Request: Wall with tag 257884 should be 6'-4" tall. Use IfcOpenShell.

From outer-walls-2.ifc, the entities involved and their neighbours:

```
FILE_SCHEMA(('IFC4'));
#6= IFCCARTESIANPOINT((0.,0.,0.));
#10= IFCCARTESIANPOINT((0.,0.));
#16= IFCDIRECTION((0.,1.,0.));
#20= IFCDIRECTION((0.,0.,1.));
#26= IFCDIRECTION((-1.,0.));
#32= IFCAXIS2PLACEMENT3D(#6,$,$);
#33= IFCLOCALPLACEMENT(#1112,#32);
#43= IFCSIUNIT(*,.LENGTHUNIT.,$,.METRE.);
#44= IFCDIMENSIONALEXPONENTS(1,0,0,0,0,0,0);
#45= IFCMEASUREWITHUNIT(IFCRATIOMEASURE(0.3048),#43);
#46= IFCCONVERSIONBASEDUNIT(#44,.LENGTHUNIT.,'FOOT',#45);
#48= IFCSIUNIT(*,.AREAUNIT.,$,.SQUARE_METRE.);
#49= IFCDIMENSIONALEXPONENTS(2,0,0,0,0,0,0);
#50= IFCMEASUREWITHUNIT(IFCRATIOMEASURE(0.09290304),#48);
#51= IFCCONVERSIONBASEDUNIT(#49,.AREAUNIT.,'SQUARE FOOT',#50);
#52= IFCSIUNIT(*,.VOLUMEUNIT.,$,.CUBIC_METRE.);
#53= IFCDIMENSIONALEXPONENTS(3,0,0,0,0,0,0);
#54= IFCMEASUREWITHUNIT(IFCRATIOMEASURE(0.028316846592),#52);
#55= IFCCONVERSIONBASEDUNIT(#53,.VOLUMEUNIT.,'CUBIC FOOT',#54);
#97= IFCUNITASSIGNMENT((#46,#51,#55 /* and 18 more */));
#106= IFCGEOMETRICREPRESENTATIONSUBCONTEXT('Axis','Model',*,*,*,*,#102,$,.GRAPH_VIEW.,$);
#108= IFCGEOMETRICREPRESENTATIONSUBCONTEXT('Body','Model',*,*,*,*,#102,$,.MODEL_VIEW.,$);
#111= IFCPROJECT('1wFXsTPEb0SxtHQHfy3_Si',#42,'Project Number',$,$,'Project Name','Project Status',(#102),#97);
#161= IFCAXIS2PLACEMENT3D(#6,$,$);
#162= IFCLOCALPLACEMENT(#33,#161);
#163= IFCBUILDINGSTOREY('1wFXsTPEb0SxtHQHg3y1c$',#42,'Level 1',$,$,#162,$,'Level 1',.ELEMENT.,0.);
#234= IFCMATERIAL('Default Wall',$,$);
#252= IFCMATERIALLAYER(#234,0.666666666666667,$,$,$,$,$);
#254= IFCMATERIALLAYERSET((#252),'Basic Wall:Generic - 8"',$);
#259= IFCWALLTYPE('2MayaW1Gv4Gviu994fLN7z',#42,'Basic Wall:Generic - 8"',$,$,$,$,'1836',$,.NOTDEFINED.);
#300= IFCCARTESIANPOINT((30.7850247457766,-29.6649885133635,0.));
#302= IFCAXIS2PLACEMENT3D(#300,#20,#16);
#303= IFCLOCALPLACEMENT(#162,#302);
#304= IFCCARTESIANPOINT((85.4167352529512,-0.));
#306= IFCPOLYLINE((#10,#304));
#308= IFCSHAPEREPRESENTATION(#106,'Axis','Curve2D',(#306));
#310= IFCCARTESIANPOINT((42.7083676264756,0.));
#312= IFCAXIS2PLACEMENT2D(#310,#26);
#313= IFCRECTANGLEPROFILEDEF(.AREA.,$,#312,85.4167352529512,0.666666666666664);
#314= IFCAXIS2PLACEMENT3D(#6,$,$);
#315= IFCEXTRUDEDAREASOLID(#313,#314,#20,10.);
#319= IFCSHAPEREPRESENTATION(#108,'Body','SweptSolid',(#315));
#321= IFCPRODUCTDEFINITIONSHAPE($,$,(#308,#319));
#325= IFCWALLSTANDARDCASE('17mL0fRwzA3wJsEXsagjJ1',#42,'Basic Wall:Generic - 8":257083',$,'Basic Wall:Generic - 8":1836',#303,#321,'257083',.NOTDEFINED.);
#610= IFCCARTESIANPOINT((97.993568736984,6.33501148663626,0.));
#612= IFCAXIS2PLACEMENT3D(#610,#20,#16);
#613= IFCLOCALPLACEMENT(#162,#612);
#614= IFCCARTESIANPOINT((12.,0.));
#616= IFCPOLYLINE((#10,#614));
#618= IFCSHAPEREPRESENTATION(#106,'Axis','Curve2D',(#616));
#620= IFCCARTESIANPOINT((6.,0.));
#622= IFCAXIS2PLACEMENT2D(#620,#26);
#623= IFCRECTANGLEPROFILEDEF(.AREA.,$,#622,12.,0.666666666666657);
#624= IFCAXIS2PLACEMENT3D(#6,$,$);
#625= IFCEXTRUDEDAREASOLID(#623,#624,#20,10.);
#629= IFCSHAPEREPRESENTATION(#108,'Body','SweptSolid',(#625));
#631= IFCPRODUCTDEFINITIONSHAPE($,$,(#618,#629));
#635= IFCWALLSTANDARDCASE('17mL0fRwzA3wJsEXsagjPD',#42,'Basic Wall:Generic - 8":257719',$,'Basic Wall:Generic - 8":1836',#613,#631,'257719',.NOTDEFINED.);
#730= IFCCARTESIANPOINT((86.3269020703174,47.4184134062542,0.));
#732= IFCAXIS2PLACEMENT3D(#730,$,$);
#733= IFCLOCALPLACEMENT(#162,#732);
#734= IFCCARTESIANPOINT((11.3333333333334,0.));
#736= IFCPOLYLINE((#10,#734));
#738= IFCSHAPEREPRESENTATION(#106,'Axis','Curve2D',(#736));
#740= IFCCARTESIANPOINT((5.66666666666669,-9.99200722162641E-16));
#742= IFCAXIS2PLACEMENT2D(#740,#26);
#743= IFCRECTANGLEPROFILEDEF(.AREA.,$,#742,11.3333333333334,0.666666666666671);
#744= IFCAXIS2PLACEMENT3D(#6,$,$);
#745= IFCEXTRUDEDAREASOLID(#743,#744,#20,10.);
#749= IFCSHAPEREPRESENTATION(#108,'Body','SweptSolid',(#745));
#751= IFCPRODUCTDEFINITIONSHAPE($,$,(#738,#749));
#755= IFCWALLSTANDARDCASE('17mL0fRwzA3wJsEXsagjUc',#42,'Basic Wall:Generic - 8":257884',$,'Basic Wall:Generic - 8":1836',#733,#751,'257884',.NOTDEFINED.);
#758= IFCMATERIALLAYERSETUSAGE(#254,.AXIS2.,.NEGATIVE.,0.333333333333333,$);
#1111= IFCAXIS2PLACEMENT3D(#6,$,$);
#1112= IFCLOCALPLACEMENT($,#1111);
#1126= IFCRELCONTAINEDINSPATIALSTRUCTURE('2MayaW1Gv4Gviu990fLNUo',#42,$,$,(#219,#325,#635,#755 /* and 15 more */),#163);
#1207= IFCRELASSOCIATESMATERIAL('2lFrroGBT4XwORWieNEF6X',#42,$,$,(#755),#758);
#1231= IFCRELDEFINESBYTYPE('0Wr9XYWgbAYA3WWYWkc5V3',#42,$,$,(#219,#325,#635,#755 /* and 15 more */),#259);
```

```python
import ifcopenshell
import ifcopenshell.geom
import ifcopenshell.util.representation
import ifcopenshell.util.shape
import ifcopenshell.util.unit

model = ifcopenshell.open("outer-walls-2.ifc")
unit_scale = ifcopenshell.util.unit.calculate_unit_scale(model)
settings = ifcopenshell.geom.settings()


def volume(element):
    """Net volume in cubic metres, openings subtracted."""
    shape = ifcopenshell.geom.create_shape(settings, element)
    return ifcopenshell.util.shape.get_volume(shape.geometry)


wall = model.by_id(755)
before = volume(wall)

body = ifcopenshell.util.representation.get_representation(wall, "Model", "Body")
solid = body.Items[0]
old_height = solid.Depth
solid.Depth = 76 * 0.0254 / unit_scale
after = volume(wall)

print(f"height {old_height:g} -> {solid.Depth:g}, volume {before:.3f} -> {after:.3f} m3")

model.write("outer-walls-2_v2.ifc")
```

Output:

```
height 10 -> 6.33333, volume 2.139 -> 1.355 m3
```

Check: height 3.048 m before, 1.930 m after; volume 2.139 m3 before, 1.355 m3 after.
